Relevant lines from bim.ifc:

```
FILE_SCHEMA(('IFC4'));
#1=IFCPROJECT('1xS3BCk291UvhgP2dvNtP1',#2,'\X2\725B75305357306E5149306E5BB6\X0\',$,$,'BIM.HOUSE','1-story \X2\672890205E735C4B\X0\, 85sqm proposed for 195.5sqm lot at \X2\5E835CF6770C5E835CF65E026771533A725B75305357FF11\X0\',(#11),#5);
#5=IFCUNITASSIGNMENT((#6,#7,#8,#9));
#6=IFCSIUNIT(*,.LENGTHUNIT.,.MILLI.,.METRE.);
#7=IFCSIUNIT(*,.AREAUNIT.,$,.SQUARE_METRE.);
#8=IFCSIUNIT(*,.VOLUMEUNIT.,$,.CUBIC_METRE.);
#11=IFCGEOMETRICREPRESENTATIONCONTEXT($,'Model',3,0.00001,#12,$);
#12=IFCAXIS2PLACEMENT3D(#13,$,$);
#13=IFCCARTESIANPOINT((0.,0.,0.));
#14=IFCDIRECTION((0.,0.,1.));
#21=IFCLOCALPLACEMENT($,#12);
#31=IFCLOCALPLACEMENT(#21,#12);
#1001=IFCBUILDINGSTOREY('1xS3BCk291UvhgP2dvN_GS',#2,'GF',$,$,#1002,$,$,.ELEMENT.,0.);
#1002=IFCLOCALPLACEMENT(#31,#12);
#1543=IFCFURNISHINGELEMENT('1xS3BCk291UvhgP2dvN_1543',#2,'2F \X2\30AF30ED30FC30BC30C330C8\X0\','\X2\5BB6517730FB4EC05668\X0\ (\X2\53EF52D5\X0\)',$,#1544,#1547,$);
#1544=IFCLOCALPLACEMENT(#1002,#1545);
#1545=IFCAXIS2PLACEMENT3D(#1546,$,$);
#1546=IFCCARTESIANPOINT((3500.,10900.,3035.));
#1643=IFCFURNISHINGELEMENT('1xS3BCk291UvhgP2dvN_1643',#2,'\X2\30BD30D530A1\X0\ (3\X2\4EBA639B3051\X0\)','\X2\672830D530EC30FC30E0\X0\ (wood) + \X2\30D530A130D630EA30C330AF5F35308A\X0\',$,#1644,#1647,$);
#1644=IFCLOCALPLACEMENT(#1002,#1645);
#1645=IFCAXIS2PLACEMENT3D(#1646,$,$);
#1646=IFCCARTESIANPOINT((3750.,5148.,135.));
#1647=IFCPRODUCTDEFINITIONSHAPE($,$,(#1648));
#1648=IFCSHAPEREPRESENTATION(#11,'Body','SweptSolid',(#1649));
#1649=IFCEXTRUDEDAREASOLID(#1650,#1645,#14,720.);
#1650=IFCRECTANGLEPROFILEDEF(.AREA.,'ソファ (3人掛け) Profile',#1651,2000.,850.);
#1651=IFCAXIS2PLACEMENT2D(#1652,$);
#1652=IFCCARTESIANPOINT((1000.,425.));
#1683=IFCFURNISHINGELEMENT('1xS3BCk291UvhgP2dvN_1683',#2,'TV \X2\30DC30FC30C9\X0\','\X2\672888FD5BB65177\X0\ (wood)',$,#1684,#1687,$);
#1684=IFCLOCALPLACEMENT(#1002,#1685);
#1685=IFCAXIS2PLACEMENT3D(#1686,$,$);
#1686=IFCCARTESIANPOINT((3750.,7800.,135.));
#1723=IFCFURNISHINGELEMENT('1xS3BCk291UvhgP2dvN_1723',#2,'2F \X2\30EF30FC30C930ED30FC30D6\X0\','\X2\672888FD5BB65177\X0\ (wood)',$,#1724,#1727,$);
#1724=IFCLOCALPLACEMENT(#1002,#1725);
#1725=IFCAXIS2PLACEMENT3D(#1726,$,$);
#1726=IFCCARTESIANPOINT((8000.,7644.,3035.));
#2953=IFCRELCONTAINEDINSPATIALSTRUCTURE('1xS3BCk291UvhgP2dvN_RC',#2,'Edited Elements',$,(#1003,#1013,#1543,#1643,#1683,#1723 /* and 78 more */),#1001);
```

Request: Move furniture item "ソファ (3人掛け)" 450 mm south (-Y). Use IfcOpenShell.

```python
import ifcopenshell
import ifcopenshell.api.geometry
import ifcopenshell.util.placement
import ifcopenshell.util.unit

model = ifcopenshell.open("bim.ifc")
unit_scale = ifcopenshell.util.unit.calculate_unit_scale(model)

item = model.by_id(1643)
matrix = ifcopenshell.util.placement.get_local_placement(item.ObjectPlacement)
matrix[1, 3] -= 0.45 / unit_scale
ifcopenshell.api.geometry.edit_object_placement(model, product=item, matrix=matrix, is_si=False)

print(ifcopenshell.util.placement.get_local_placement(item.ObjectPlacement).round(3) + 0.0)

model.write("bim_edited.ifc")
```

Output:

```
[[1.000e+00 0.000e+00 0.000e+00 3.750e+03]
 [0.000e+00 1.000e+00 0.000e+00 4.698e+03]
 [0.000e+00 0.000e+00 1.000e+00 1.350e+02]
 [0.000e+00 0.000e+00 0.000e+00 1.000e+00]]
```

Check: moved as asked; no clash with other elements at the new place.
